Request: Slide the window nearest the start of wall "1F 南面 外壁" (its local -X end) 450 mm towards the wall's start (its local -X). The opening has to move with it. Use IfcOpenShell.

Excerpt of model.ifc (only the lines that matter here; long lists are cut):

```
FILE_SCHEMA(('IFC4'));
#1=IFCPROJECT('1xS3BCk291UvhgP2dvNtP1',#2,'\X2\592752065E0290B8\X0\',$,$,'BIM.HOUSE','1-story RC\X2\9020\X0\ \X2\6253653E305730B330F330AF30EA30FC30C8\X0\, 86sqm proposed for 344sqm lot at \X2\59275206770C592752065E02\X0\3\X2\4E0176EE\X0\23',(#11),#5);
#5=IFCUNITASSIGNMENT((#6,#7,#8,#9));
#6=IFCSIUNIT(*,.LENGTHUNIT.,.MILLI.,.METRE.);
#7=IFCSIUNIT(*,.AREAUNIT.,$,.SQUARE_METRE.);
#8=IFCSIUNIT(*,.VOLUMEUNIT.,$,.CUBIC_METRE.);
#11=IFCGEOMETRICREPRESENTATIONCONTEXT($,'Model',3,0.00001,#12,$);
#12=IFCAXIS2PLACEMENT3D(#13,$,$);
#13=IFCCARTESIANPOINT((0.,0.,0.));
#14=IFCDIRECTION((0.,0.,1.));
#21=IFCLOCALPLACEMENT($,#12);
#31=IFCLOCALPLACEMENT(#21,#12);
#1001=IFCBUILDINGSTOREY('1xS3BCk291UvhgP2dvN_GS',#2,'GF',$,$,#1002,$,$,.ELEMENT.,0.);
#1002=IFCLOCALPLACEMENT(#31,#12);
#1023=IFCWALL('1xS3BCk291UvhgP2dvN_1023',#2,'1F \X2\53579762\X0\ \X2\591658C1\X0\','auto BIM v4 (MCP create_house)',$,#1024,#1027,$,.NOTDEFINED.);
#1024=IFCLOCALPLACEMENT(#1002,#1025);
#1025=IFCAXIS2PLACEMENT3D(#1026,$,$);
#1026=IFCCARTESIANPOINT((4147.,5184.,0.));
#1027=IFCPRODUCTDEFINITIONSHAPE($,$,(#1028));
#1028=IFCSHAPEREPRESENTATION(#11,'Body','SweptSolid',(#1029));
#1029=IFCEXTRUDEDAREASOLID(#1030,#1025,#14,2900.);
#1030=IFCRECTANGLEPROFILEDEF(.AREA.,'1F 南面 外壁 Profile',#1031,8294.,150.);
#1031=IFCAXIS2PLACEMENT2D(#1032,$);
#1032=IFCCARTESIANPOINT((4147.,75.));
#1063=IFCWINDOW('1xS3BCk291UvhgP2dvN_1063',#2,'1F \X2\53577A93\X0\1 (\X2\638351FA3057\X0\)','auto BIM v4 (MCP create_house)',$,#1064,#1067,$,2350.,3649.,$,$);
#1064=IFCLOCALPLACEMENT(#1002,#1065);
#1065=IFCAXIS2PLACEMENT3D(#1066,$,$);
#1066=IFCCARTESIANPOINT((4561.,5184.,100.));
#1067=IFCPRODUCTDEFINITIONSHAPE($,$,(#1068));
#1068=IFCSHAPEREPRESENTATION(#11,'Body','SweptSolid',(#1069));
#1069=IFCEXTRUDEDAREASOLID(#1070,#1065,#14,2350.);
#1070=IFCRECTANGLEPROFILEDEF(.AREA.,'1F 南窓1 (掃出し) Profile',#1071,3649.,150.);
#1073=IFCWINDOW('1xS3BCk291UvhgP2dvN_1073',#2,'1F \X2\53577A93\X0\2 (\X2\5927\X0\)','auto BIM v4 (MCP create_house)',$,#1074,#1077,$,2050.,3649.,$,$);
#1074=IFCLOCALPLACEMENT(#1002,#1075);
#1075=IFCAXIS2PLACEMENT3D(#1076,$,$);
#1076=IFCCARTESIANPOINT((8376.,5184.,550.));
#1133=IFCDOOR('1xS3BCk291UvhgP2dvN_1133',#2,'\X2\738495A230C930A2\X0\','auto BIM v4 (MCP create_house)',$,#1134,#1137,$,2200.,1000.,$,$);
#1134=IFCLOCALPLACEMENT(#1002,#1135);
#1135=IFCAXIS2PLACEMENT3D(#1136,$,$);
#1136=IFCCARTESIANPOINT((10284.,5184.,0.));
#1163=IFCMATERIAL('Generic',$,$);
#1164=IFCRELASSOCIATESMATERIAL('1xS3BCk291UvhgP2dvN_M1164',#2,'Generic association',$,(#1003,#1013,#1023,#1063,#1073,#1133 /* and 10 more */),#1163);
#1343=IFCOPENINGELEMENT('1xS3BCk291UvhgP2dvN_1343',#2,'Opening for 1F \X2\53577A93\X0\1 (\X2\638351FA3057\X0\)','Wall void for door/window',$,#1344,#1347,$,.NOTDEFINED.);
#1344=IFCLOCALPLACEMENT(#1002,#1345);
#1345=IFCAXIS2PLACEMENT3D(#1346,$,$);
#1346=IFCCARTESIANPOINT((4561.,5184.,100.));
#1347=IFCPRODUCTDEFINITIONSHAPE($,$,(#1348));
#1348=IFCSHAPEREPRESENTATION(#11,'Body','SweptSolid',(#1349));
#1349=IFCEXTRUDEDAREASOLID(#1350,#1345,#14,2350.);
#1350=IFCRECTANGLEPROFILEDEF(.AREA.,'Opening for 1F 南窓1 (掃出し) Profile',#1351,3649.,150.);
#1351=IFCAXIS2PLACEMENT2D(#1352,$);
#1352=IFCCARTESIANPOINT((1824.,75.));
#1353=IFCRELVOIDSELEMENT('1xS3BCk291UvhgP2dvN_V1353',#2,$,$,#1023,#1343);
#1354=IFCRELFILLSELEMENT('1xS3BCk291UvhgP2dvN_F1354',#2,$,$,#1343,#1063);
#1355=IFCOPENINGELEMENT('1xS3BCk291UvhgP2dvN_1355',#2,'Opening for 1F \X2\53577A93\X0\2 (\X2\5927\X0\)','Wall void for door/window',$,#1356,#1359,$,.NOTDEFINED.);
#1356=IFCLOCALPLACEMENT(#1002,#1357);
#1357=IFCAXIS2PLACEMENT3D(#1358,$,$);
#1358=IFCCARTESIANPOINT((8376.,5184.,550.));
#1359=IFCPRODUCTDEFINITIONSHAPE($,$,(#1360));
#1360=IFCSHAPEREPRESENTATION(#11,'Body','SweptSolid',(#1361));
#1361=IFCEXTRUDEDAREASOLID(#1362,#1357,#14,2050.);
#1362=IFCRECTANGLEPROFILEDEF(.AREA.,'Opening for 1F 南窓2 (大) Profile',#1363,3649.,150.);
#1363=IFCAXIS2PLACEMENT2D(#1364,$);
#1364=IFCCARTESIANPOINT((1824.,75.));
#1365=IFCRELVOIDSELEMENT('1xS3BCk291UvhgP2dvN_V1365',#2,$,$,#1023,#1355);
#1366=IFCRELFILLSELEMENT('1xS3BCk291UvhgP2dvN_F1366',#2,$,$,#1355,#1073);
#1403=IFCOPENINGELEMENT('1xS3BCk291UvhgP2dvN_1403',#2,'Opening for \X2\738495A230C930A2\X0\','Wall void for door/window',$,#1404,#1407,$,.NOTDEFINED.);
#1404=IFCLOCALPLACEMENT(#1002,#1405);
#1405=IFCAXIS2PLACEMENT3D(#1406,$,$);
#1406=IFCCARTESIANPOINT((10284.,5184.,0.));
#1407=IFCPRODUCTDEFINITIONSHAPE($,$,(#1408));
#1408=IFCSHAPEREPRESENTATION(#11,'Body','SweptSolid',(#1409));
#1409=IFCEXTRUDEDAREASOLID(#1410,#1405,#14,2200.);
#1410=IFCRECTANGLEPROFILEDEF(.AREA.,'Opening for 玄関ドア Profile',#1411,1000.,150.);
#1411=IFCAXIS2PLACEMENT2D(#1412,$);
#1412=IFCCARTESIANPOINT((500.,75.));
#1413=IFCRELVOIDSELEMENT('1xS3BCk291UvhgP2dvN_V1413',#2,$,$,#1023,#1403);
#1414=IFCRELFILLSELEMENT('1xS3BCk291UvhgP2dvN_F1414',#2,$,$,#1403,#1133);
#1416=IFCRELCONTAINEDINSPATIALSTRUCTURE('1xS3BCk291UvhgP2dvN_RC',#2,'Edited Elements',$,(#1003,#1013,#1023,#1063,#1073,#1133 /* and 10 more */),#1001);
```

```python
import ifcopenshell
import ifcopenshell.api.geometry
import ifcopenshell.util.placement
import ifcopenshell.util.unit

model = ifcopenshell.open("model.ifc")
unit_scale = ifcopenshell.util.unit.calculate_unit_scale(model)

window = model.by_guid("1xS3BCk291UvhgP2dvN_1063")
opening = window.FillsVoids[0].RelatingOpeningElement
wall = opening.VoidsElements[0].RelatingBuildingElement

wall_matrix = ifcopenshell.util.placement.get_local_placement(wall.ObjectPlacement)
shift = wall_matrix[:3, 0] * -0.45 / unit_scale
before = ifcopenshell.util.placement.get_local_placement(window.ObjectPlacement)[:3, 3].copy()

# The window is not placed relative to its opening, so move both.
for product in (opening, window):
    matrix = ifcopenshell.util.placement.get_local_placement(product.ObjectPlacement)
    matrix[:3, 3] += shift
    ifcopenshell.api.geometry.edit_object_placement(model, product=product, matrix=matrix, is_si=False)

after = ifcopenshell.util.placement.get_local_placement(window.ObjectPlacement)[:3, 3]
print("window moved by", (after - before).round(3) + 0.0)

model.write("model-out.ifc")
```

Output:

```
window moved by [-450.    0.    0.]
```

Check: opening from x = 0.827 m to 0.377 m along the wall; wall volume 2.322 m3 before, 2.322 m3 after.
